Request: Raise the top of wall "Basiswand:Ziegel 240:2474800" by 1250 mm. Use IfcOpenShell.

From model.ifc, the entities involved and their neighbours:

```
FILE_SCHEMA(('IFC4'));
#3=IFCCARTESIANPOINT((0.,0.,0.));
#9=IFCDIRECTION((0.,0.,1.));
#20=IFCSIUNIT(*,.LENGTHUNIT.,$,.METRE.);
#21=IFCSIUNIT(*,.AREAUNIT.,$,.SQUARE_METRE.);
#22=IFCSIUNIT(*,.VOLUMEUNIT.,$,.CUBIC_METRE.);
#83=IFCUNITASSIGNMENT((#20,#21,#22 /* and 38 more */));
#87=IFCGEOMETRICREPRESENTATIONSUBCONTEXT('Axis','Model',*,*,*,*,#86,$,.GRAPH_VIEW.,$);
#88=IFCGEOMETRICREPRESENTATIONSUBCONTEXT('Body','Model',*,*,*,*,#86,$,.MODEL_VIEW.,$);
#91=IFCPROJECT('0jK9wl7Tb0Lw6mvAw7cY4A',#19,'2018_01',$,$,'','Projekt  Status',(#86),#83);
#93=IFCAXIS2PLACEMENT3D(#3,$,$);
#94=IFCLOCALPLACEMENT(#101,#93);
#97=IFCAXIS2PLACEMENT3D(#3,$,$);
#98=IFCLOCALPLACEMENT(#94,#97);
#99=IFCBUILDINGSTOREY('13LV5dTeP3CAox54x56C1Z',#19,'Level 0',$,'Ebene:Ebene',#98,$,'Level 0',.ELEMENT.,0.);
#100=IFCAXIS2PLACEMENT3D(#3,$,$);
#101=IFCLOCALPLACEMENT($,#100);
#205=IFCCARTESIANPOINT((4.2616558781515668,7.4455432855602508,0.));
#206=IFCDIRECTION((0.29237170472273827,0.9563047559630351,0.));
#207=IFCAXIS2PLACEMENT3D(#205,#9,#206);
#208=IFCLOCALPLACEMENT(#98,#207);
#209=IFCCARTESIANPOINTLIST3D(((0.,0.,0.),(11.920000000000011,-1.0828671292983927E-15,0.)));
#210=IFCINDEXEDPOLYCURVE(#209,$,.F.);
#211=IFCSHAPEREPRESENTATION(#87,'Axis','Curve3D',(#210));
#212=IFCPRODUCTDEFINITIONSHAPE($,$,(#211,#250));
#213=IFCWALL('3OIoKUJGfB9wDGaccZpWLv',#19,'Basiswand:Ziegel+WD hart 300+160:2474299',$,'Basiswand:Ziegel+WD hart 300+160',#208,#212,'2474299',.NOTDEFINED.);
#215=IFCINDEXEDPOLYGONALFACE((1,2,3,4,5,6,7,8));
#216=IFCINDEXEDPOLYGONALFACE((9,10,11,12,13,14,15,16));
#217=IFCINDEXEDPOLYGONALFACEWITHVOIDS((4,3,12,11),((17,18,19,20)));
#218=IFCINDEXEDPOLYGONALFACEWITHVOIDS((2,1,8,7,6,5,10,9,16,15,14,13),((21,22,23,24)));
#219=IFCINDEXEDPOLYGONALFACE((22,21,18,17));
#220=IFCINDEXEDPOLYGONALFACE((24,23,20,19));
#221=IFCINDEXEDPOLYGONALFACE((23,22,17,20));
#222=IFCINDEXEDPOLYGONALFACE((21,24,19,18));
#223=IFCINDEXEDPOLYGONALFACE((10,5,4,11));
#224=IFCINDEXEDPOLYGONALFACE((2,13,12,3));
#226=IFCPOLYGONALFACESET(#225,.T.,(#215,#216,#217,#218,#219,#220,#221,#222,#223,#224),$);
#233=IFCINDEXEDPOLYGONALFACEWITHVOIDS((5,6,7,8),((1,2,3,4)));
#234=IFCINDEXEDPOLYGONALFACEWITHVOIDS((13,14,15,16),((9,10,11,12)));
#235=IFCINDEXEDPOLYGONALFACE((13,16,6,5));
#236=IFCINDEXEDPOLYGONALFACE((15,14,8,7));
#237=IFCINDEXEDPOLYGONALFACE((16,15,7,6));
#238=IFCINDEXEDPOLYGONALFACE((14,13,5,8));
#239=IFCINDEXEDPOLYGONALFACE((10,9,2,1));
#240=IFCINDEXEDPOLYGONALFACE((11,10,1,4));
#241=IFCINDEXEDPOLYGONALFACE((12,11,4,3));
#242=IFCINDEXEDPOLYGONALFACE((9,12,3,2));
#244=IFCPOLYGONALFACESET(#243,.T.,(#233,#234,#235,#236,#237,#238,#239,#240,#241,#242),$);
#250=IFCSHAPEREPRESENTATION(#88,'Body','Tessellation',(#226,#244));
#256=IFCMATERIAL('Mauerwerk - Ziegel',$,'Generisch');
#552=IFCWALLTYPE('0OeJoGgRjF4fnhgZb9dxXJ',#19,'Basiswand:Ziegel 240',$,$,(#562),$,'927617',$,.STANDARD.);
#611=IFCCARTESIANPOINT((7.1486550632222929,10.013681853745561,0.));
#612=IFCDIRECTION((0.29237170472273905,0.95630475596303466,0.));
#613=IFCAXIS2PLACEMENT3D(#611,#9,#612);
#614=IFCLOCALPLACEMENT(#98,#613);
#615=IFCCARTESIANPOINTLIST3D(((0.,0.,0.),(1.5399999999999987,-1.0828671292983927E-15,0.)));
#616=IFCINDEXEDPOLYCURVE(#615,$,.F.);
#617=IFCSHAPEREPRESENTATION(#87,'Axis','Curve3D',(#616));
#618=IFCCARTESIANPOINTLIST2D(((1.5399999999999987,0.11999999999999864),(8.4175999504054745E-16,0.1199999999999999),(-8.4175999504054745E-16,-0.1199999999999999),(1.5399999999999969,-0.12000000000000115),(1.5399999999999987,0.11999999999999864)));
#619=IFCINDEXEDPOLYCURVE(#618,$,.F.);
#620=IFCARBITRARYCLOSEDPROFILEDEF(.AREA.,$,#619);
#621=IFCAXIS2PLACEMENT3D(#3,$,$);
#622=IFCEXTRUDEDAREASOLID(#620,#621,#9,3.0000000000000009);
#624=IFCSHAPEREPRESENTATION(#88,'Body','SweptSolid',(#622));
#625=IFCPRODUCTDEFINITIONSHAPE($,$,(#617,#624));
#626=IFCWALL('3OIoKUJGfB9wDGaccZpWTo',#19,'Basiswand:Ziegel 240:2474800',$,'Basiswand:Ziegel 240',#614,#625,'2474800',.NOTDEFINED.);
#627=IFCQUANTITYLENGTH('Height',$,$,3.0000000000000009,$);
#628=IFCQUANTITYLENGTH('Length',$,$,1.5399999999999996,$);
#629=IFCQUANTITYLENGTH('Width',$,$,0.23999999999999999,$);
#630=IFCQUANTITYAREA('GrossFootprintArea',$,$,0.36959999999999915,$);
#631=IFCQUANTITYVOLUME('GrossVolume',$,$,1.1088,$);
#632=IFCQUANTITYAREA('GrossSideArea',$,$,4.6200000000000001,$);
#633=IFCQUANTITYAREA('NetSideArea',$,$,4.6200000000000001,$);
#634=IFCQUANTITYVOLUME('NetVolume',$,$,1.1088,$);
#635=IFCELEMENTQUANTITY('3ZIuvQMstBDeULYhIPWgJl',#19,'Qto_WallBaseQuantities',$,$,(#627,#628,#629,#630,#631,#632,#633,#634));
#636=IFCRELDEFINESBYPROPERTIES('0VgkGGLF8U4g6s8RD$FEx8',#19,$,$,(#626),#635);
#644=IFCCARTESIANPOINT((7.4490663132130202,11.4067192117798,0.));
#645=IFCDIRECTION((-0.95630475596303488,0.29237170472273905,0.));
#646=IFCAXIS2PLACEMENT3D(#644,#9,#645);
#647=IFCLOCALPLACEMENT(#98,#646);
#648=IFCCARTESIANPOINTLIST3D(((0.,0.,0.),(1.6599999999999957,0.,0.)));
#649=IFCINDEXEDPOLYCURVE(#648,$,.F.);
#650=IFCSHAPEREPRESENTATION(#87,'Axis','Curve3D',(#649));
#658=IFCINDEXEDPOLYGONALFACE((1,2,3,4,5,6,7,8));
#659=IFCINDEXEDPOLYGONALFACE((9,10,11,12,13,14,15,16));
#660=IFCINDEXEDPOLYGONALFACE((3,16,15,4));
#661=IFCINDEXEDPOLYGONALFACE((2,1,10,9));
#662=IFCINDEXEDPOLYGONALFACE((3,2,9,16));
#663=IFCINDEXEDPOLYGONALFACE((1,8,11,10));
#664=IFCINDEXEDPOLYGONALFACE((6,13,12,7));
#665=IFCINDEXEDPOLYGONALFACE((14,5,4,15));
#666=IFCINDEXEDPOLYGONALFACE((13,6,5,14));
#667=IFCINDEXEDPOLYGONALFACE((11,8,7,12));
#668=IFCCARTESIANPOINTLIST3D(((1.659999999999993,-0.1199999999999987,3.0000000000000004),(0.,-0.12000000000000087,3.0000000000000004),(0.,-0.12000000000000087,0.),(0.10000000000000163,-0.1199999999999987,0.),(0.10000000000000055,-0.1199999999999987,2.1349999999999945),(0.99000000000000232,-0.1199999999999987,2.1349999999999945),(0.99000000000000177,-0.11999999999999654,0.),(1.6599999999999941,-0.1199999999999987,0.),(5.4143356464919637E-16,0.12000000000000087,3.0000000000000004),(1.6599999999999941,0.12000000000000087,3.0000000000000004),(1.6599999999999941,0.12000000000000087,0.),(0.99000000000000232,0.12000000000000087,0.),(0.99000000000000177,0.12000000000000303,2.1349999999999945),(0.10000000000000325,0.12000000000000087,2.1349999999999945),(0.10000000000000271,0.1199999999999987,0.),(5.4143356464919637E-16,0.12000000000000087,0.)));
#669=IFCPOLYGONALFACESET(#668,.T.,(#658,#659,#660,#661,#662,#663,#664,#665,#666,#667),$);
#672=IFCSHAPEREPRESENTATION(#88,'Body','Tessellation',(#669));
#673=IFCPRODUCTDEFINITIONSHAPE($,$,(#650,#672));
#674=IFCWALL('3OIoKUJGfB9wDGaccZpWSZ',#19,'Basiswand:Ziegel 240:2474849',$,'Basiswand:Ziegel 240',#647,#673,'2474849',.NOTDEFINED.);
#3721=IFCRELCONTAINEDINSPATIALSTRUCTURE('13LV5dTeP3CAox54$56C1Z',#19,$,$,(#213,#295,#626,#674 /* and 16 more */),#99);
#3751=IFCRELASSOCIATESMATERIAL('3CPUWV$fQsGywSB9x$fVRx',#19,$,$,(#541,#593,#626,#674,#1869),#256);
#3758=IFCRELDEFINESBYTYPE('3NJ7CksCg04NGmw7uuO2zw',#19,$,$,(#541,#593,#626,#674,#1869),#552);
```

```python
import ifcopenshell
import ifcopenshell.api.pset
import ifcopenshell.geom
import ifcopenshell.util.element
import ifcopenshell.util.representation
import ifcopenshell.util.shape
import ifcopenshell.util.unit

model = ifcopenshell.open("model.ifc")
unit_scale = ifcopenshell.util.unit.calculate_unit_scale(model)
area_scale = ifcopenshell.util.unit.calculate_unit_scale(model, "AREAUNIT")
volume_scale = ifcopenshell.util.unit.calculate_unit_scale(model, "VOLUMEUNIT")
settings = ifcopenshell.geom.settings()


def volume(element):
    """Net volume in cubic metres, openings subtracted."""
    shape = ifcopenshell.geom.create_shape(settings, element)
    return ifcopenshell.util.shape.get_volume(shape.geometry)


wall = model.by_guid("3OIoKUJGfB9wDGaccZpWTo")
before = volume(wall)

body = ifcopenshell.util.representation.get_representation(wall, "Model", "Body")
solid = body.Items[0]
old_height = solid.Depth
solid.Depth += 1.25 / unit_scale
after = volume(wall)
thickness = 0.24  # wall thickness in metres

# Update the stored height, areas and volumes.
qto = model.by_id(ifcopenshell.util.element.get_pset(wall, "Qto_WallBaseQuantities", should_inherit=False)["id"])
ifcopenshell.api.pset.edit_qto(model, qto=qto, properties={
    "Height": solid.Depth,
    "GrossVolume": ifcopenshell.util.element.get_pset(wall, "Qto_WallBaseQuantities", "GrossVolume") * solid.Depth / old_height,
    "GrossSideArea": ifcopenshell.util.element.get_pset(wall, "Qto_WallBaseQuantities", "GrossSideArea") * solid.Depth / old_height,
    "NetSideArea": after / thickness / area_scale,
    "NetVolume": after / volume_scale,
})

print(f"height {old_height:g} -> {solid.Depth:g}, volume {before:.3f} -> {after:.3f} m3")

model.write("model_edited.ifc")
```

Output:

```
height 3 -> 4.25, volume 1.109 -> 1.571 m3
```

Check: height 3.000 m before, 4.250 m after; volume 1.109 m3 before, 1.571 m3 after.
